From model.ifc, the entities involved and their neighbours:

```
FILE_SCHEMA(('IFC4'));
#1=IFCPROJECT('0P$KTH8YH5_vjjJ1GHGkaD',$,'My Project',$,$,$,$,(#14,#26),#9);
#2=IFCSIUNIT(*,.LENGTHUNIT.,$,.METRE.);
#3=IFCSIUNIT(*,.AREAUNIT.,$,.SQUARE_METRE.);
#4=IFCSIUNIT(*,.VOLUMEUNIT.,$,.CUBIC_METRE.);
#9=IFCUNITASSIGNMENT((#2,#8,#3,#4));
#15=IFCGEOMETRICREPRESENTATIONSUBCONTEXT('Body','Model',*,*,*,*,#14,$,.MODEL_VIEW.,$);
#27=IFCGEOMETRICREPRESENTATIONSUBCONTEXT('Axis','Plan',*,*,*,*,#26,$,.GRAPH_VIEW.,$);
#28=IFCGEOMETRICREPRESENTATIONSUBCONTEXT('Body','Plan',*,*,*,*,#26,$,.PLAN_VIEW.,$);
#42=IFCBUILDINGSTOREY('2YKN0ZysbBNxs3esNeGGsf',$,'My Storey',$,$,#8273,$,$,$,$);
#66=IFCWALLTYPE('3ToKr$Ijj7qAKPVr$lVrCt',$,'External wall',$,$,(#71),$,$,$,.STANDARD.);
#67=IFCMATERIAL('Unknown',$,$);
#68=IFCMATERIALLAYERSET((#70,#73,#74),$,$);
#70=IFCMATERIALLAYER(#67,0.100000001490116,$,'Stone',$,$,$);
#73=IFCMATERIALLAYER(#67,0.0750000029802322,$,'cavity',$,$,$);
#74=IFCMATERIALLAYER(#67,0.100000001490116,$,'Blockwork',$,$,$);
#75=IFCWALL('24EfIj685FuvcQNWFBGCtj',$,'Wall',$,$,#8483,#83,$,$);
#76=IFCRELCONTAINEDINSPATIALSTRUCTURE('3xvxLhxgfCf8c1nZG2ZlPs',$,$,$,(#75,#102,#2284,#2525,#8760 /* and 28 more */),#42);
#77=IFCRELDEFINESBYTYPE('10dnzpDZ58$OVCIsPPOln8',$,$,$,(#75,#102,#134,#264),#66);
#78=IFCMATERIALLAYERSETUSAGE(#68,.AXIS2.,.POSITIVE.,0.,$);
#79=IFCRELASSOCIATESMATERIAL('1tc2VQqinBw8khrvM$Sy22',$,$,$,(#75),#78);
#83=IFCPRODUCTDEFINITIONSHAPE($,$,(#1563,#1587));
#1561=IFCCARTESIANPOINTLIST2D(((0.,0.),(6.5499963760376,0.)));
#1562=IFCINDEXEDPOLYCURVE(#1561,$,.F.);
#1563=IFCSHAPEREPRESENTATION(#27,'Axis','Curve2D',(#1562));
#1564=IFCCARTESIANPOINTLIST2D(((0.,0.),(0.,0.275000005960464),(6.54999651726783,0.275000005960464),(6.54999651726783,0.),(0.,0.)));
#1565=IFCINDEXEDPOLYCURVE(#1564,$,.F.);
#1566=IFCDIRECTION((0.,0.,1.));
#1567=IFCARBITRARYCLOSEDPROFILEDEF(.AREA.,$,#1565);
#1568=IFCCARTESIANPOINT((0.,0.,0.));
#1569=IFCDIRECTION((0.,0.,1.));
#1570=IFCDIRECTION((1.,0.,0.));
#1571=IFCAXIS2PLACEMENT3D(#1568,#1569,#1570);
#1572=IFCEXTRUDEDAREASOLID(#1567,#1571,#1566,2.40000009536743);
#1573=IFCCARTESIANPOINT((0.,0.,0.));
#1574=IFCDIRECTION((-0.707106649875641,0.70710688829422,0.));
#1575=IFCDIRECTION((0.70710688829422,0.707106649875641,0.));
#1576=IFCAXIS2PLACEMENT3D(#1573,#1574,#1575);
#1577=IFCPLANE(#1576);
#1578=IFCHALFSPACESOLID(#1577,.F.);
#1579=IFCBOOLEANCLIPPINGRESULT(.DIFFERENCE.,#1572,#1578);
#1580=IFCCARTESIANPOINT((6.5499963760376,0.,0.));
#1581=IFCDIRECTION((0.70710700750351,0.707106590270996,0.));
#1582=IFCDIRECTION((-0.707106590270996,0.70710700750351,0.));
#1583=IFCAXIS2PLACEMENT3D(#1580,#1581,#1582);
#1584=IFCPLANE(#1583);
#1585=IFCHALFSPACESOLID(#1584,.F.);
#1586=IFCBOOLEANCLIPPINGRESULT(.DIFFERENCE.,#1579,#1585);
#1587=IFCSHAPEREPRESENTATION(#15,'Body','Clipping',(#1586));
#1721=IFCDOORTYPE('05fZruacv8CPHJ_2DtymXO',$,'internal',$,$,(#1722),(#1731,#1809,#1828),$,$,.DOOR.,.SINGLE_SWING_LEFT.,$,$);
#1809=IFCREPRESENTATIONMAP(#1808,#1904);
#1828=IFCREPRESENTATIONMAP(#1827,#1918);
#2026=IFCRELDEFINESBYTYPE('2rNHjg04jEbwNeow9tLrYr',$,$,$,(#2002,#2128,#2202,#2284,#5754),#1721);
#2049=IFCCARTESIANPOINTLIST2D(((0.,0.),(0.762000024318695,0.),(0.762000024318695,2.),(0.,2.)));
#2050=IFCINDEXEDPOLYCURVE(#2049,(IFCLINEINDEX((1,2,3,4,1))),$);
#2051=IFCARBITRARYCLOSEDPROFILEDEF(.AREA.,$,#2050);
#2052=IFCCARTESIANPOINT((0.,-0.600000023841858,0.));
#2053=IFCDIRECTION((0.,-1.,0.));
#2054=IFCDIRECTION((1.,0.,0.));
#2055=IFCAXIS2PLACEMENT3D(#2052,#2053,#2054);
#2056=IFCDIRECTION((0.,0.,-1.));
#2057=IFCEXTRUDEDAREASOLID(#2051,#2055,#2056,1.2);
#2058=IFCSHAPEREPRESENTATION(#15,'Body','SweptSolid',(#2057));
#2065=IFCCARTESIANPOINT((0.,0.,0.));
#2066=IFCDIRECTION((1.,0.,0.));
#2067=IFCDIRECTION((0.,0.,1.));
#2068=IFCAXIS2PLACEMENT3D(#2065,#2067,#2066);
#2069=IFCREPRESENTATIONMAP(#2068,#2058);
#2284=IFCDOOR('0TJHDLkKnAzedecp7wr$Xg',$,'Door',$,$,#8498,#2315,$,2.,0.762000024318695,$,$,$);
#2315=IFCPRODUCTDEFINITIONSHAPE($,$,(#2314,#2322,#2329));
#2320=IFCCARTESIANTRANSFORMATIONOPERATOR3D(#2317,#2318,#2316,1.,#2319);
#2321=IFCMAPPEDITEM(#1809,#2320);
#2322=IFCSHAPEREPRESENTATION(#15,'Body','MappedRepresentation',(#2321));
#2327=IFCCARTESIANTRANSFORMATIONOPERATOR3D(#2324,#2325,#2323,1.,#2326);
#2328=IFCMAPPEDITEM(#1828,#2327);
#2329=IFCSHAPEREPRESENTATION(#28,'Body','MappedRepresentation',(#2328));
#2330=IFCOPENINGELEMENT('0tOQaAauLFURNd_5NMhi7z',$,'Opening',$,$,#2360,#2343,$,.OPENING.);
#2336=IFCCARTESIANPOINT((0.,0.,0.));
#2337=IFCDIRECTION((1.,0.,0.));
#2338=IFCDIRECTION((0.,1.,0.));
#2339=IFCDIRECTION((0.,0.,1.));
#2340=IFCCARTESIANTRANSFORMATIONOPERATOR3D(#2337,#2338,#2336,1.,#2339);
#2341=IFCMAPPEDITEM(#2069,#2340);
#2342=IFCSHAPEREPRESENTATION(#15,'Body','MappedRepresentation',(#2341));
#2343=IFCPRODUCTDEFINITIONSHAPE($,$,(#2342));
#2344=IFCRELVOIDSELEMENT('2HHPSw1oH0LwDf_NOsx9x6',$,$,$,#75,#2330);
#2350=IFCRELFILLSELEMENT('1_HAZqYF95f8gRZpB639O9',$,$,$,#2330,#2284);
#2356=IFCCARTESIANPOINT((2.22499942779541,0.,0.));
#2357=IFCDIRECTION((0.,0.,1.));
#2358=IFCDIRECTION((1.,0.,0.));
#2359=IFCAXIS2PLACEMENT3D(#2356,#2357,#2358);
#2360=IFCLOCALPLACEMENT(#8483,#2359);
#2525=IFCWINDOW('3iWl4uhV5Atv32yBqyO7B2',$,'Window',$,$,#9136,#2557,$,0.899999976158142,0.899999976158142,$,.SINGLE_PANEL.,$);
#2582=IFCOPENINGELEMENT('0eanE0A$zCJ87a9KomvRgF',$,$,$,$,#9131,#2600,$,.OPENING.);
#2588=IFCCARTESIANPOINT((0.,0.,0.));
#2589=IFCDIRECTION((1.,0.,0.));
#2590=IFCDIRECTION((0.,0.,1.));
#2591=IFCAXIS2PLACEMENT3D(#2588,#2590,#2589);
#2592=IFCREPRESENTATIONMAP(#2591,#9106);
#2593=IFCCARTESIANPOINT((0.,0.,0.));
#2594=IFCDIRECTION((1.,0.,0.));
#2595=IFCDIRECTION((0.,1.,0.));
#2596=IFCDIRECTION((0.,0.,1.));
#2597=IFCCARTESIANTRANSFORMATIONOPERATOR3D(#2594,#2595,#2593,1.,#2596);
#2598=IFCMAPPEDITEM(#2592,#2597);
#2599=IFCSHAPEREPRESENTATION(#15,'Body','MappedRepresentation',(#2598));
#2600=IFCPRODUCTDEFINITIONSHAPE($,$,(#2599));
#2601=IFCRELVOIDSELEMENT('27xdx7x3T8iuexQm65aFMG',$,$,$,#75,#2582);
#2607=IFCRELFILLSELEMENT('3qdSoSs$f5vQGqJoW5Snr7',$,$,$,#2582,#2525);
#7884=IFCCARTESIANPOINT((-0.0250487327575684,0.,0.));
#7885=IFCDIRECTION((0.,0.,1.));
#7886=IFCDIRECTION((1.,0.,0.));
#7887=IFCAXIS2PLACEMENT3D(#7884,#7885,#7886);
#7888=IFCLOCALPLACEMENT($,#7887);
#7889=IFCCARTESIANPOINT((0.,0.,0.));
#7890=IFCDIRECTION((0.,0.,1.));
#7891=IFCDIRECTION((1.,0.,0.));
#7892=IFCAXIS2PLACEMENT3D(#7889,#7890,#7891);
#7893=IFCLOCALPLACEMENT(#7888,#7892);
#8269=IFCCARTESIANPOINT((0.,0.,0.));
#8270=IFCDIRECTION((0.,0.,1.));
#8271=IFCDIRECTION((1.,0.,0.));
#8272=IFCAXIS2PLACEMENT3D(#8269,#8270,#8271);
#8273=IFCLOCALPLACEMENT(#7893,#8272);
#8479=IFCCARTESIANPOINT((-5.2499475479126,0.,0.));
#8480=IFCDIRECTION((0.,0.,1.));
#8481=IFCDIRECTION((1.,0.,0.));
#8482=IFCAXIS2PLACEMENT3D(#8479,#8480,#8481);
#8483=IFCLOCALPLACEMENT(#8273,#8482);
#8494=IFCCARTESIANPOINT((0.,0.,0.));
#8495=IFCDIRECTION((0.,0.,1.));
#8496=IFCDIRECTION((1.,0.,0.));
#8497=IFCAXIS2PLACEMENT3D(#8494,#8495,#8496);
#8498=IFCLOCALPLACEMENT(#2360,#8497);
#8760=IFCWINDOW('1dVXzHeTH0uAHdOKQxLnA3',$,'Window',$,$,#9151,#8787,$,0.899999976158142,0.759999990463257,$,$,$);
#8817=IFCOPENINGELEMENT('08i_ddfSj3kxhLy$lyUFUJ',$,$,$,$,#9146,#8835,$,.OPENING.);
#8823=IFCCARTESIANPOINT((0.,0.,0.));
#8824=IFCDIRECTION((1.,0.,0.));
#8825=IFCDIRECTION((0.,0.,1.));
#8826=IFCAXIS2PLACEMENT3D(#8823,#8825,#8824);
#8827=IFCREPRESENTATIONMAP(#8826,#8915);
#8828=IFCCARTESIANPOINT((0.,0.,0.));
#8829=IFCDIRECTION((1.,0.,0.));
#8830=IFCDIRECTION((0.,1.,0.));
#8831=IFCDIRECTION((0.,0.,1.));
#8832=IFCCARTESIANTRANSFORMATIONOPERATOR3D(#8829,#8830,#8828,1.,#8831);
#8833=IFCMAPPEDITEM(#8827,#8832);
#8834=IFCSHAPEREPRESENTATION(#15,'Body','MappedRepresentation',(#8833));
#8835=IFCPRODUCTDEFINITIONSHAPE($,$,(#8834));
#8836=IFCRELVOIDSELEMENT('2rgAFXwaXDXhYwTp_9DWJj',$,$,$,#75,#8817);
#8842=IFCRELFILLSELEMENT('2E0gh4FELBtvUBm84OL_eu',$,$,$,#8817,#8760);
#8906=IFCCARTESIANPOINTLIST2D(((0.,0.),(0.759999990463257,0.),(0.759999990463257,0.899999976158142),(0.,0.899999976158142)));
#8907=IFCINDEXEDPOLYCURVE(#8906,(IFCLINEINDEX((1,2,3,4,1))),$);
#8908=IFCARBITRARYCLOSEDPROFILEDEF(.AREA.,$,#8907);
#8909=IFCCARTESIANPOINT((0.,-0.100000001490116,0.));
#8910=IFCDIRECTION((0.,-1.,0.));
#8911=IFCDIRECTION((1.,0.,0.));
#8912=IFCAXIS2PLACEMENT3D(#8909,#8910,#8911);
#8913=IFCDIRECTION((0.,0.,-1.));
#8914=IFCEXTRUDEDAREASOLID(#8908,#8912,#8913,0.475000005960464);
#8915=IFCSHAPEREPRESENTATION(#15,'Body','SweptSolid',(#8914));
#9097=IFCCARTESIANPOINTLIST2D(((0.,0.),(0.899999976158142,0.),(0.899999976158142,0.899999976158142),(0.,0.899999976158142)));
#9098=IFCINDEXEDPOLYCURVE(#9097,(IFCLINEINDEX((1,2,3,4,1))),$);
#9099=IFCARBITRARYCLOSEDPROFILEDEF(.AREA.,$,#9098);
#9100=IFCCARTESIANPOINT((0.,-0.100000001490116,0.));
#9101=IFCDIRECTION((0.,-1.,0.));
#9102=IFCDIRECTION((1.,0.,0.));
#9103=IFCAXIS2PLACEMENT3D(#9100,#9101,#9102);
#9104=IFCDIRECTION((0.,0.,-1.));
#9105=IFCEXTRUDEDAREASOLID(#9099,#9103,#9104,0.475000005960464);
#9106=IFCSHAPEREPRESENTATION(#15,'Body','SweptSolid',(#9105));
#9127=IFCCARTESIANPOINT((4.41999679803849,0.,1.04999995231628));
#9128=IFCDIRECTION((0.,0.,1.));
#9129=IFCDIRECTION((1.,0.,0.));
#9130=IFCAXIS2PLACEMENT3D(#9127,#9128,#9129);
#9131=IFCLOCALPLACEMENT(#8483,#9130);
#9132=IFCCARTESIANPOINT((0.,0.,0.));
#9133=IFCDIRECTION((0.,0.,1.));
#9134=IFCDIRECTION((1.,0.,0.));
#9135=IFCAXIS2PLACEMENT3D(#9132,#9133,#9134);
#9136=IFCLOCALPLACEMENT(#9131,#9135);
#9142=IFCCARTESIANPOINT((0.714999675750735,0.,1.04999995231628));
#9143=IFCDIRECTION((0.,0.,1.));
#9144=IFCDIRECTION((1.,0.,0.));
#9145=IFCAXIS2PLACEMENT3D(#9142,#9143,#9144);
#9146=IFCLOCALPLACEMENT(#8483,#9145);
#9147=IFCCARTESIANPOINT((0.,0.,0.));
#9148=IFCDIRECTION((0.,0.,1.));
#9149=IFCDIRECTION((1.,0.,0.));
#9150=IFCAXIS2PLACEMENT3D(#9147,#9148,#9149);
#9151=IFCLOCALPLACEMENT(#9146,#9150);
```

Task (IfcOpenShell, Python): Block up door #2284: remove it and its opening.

```python
import ifcopenshell
import ifcopenshell.api.feature
import ifcopenshell.api.root
import ifcopenshell.geom
import ifcopenshell.util.shape

model = ifcopenshell.open("model.ifc")
settings = ifcopenshell.geom.settings()


def volume(element):
    """Net volume in cubic metres, openings subtracted."""
    shape = ifcopenshell.geom.create_shape(settings, element)
    return ifcopenshell.util.shape.get_volume(shape.geometry)


door = model.by_guid("0TJHDLkKnAzedecp7wr$Xg")
opening = door.FillsVoids[0].RelatingOpeningElement
wall = opening.VoidsElements[0].RelatingBuildingElement
before = volume(wall)

ifcopenshell.api.root.remove_product(model, product=door)
ifcopenshell.api.feature.remove_feature(model, feature=opening)

after = volume(wall)

print(f"wall volume {before:.3f} -> {after:.3f} m3")

model.write("model_v2.ifc")
```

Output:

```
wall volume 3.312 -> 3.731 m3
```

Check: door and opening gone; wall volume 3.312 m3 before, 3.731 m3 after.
